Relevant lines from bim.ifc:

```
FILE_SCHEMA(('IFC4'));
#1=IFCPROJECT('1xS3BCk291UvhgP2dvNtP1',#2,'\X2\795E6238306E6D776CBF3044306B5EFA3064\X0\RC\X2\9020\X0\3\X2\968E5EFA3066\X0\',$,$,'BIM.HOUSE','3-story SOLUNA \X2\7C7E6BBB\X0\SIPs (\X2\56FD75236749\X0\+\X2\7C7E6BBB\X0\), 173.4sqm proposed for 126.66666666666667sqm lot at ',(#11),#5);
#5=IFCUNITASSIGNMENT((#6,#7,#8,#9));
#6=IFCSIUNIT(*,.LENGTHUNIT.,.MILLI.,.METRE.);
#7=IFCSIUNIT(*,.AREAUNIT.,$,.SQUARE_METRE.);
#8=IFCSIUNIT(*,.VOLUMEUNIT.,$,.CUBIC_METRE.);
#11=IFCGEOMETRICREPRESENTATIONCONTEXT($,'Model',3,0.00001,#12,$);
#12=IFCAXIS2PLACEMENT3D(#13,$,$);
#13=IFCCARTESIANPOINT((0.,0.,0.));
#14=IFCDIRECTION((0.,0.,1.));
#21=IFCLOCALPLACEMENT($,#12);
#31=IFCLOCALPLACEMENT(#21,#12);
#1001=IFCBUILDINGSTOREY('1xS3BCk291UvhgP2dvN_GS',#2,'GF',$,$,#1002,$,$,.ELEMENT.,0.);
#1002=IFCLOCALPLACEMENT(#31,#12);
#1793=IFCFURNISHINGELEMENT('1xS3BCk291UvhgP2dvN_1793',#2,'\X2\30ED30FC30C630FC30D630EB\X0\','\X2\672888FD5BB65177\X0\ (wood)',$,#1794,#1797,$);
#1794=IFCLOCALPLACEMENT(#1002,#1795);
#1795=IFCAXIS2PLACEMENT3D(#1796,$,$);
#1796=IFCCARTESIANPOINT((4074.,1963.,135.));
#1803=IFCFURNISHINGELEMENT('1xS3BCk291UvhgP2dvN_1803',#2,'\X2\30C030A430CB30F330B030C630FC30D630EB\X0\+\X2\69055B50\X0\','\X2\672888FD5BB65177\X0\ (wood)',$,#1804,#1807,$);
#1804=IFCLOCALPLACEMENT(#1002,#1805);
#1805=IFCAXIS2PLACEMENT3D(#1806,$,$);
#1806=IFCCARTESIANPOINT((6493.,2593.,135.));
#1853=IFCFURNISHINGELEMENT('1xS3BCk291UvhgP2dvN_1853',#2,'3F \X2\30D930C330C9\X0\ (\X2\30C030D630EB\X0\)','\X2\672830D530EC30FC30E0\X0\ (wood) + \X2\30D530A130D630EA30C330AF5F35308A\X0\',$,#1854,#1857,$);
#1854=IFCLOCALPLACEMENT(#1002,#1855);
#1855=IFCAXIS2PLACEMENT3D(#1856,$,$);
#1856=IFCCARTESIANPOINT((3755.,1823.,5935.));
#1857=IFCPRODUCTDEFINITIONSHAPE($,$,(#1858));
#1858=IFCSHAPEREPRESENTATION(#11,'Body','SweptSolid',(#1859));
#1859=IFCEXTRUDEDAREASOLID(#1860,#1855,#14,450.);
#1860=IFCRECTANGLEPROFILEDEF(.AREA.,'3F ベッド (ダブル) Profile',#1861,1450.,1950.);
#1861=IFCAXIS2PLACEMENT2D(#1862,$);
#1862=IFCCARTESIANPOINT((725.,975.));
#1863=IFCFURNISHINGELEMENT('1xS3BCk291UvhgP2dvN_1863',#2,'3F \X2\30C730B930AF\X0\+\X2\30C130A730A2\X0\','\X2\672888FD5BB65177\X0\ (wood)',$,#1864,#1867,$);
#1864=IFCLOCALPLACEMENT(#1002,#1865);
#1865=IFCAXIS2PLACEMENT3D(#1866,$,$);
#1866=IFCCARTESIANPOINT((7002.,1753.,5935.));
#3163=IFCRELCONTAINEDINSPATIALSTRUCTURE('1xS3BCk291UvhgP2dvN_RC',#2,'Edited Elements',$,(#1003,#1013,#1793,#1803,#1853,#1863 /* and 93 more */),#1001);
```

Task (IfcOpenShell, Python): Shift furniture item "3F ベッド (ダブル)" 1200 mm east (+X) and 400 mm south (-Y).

```python
import ifcopenshell
import ifcopenshell.api.geometry
import ifcopenshell.util.placement

model = ifcopenshell.open("bim.ifc")

item = model.by_guid("1xS3BCk291UvhgP2dvN_1853")
matrix = ifcopenshell.util.placement.get_local_placement(item.ObjectPlacement)
matrix[0, 3] += 1200.0
matrix[1, 3] -= 400.0
ifcopenshell.api.geometry.edit_object_placement(model, product=item, matrix=matrix, is_si=False)

print(ifcopenshell.util.placement.get_local_placement(item.ObjectPlacement).round(3) + 0.0)

model.write("bim-out.ifc")
```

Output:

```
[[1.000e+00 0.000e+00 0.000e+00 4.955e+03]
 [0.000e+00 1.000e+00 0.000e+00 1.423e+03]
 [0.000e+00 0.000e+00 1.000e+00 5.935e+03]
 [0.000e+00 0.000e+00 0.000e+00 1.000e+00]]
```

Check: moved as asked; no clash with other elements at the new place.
